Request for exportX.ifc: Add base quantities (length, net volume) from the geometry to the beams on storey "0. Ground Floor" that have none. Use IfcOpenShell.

First a look at what the model holds.

```python
import ifcopenshell
import ifcopenshell.util.element
import ifcopenshell.util.unit

model = ifcopenshell.open("exportX.ifc")
print(model.schema)
for unit_type in ("LENGTHUNIT", "AREAUNIT", "VOLUMEUNIT"):
    print(unit_type, ifcopenshell.util.unit.calculate_unit_scale(model, unit_type))
storey = next(s for s in model.by_type("IfcBuildingStorey") if s.Name == "0. Ground Floor")
beams = [e for e in ifcopenshell.util.element.get_decomposition(storey) if e.is_a("IfcBeam")]
for e in sorted(beams, key=lambda e: e.id()):
    print(e.id(), e.is_a(), e.Name, list(ifcopenshell.util.element.get_psets(e, qtos_only=True)), sep=" | ")
```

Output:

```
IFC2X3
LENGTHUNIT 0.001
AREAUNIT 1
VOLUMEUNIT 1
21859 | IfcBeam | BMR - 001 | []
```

```python
import ifcopenshell
import ifcopenshell.api.pset
import ifcopenshell.geom
import ifcopenshell.util.element
import ifcopenshell.util.shape
import ifcopenshell.util.unit

model = ifcopenshell.open("exportX.ifc")
unit_scale = ifcopenshell.util.unit.calculate_unit_scale(model)
volume_scale = ifcopenshell.util.unit.calculate_unit_scale(model, "VOLUMEUNIT")
settings = ifcopenshell.geom.settings()

storey = next(s for s in model.by_type("IfcBuildingStorey") if s.Name == "0. Ground Floor")
beams = [e for e in ifcopenshell.util.element.get_decomposition(storey) if e.is_a("IfcBeam")]

for e in sorted(beams, key=lambda e: e.id()):
    if ifcopenshell.util.element.get_psets(e, qtos_only=True, should_inherit=False):
        continue
    # Geometry comes back in metres, in the element's own axes.
    shape = ifcopenshell.geom.create_shape(settings, e)
    values = {
        "Length": ifcopenshell.util.shape.get_max_xyz(shape.geometry) / unit_scale,
        "NetVolume": ifcopenshell.util.shape.get_volume(shape.geometry) / volume_scale,
    }
    qto = ifcopenshell.api.pset.add_qto(model, product=e, name="BaseQuantities")
    ifcopenshell.api.pset.edit_qto(model, qto=qto, properties=values)
    print(e.id(), {k: round(v, 3) for k, v in values.items()})

model.write("exportX_edited.ifc")
```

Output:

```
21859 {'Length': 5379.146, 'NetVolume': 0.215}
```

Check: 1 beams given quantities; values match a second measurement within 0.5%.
